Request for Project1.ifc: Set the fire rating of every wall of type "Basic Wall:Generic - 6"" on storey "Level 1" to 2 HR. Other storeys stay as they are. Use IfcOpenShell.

First a look at what the model holds.

```python
import ifcopenshell
import ifcopenshell.util.element

model = ifcopenshell.open("Project1.ifc")
print(model.schema)
storey = next(s for s in model.by_type("IfcBuildingStorey") if s.Name == "Level 1")
walls = [e for e in ifcopenshell.util.element.get_decomposition(storey) if e.is_a("IfcWall")]
seen = {}
for e in walls:
    element_type = ifcopenshell.util.element.get_type(e)
    key = (element_type.Name if element_type != e and element_type else None, ifcopenshell.util.element.get_pset(e, "Pset_WallCommon", "FireRating"))
    seen[key] = seen.get(key, 0) + 1
for (name, value), count in sorted(seen.items(), key=str):
    print(count, "x", name, "|", value)
```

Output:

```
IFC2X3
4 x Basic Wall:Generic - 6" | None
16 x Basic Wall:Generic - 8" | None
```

```python
import ifcopenshell
import ifcopenshell.api.pset
import ifcopenshell.util.element

model = ifcopenshell.open("Project1.ifc")

storey = next(s for s in model.by_type("IfcBuildingStorey") if s.Name == "Level 1")
walls = [e for e in ifcopenshell.util.element.get_decomposition(storey) if e.is_a("IfcWall")]

count = 0
for e in walls:
    element_type = ifcopenshell.util.element.get_type(e)
    if element_type in (None, e) or element_type.Name != 'Basic Wall:Generic - 6"':
        continue
    # add_pset returns the element's existing set when there is one.
    pset = ifcopenshell.api.pset.add_pset(model, product=e, name="Pset_WallCommon")
    ifcopenshell.api.pset.edit_pset(model, pset=pset, properties={"FireRating": "2 HR"})
    count += 1

print(count, "walls updated")

model.write("Project1_rev.ifc")
```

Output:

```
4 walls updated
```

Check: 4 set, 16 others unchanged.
